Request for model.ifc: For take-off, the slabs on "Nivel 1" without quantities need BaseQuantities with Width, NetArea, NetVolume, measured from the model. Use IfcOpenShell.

First a look at what the model holds.

```python
import ifcopenshell
import ifcopenshell.util.element
import ifcopenshell.util.unit

model = ifcopenshell.open("model.ifc")
print(model.schema)
for unit_type in ("LENGTHUNIT", "AREAUNIT", "VOLUMEUNIT"):
    print(unit_type, ifcopenshell.util.unit.calculate_unit_scale(model, unit_type))
storey = next(s for s in model.by_type("IfcBuildingStorey") if s.Name == "Nivel 1")
slabs = [e for e in ifcopenshell.util.element.get_decomposition(storey) if e.is_a("IfcSlab")]
for e in sorted(slabs, key=lambda e: e.id()):
    print(e.id(), e.is_a(), e.Name, list(ifcopenshell.util.element.get_psets(e, qtos_only=True)), sep=" | ")
```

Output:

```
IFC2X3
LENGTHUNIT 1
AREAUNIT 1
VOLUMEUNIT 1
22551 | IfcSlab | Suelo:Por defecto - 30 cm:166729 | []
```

```python
import ifcopenshell
import ifcopenshell.api.pset
import ifcopenshell.geom
import ifcopenshell.util.element
import ifcopenshell.util.shape
import ifcopenshell.util.unit

model = ifcopenshell.open("model.ifc")
unit_scale = ifcopenshell.util.unit.calculate_unit_scale(model)
area_scale = ifcopenshell.util.unit.calculate_unit_scale(model, "AREAUNIT")
volume_scale = ifcopenshell.util.unit.calculate_unit_scale(model, "VOLUMEUNIT")
settings = ifcopenshell.geom.settings()

storey = next(s for s in model.by_type("IfcBuildingStorey") if s.Name == "Nivel 1")
slabs = [e for e in ifcopenshell.util.element.get_decomposition(storey) if e.is_a("IfcSlab")]

for e in sorted(slabs, key=lambda e: e.id()):
    if ifcopenshell.util.element.get_psets(e, qtos_only=True, should_inherit=False):
        continue
    # Geometry comes back in metres, in the element's own axes.
    shape = ifcopenshell.geom.create_shape(settings, e)
    values = {
        "Width": ifcopenshell.util.shape.get_z(shape.geometry) / unit_scale,
        "NetArea": ifcopenshell.util.shape.get_footprint_area(shape.geometry) / area_scale,
        "NetVolume": ifcopenshell.util.shape.get_volume(shape.geometry) / volume_scale,
    }
    qto = ifcopenshell.api.pset.add_qto(model, product=e, name="BaseQuantities")
    ifcopenshell.api.pset.edit_qto(model, qto=qto, properties=values)
    print(e.id(), {k: round(v, 3) for k, v in values.items()})

model.write("model_updated.ifc")
```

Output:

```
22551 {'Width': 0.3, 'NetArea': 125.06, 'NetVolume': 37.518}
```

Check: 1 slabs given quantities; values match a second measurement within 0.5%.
